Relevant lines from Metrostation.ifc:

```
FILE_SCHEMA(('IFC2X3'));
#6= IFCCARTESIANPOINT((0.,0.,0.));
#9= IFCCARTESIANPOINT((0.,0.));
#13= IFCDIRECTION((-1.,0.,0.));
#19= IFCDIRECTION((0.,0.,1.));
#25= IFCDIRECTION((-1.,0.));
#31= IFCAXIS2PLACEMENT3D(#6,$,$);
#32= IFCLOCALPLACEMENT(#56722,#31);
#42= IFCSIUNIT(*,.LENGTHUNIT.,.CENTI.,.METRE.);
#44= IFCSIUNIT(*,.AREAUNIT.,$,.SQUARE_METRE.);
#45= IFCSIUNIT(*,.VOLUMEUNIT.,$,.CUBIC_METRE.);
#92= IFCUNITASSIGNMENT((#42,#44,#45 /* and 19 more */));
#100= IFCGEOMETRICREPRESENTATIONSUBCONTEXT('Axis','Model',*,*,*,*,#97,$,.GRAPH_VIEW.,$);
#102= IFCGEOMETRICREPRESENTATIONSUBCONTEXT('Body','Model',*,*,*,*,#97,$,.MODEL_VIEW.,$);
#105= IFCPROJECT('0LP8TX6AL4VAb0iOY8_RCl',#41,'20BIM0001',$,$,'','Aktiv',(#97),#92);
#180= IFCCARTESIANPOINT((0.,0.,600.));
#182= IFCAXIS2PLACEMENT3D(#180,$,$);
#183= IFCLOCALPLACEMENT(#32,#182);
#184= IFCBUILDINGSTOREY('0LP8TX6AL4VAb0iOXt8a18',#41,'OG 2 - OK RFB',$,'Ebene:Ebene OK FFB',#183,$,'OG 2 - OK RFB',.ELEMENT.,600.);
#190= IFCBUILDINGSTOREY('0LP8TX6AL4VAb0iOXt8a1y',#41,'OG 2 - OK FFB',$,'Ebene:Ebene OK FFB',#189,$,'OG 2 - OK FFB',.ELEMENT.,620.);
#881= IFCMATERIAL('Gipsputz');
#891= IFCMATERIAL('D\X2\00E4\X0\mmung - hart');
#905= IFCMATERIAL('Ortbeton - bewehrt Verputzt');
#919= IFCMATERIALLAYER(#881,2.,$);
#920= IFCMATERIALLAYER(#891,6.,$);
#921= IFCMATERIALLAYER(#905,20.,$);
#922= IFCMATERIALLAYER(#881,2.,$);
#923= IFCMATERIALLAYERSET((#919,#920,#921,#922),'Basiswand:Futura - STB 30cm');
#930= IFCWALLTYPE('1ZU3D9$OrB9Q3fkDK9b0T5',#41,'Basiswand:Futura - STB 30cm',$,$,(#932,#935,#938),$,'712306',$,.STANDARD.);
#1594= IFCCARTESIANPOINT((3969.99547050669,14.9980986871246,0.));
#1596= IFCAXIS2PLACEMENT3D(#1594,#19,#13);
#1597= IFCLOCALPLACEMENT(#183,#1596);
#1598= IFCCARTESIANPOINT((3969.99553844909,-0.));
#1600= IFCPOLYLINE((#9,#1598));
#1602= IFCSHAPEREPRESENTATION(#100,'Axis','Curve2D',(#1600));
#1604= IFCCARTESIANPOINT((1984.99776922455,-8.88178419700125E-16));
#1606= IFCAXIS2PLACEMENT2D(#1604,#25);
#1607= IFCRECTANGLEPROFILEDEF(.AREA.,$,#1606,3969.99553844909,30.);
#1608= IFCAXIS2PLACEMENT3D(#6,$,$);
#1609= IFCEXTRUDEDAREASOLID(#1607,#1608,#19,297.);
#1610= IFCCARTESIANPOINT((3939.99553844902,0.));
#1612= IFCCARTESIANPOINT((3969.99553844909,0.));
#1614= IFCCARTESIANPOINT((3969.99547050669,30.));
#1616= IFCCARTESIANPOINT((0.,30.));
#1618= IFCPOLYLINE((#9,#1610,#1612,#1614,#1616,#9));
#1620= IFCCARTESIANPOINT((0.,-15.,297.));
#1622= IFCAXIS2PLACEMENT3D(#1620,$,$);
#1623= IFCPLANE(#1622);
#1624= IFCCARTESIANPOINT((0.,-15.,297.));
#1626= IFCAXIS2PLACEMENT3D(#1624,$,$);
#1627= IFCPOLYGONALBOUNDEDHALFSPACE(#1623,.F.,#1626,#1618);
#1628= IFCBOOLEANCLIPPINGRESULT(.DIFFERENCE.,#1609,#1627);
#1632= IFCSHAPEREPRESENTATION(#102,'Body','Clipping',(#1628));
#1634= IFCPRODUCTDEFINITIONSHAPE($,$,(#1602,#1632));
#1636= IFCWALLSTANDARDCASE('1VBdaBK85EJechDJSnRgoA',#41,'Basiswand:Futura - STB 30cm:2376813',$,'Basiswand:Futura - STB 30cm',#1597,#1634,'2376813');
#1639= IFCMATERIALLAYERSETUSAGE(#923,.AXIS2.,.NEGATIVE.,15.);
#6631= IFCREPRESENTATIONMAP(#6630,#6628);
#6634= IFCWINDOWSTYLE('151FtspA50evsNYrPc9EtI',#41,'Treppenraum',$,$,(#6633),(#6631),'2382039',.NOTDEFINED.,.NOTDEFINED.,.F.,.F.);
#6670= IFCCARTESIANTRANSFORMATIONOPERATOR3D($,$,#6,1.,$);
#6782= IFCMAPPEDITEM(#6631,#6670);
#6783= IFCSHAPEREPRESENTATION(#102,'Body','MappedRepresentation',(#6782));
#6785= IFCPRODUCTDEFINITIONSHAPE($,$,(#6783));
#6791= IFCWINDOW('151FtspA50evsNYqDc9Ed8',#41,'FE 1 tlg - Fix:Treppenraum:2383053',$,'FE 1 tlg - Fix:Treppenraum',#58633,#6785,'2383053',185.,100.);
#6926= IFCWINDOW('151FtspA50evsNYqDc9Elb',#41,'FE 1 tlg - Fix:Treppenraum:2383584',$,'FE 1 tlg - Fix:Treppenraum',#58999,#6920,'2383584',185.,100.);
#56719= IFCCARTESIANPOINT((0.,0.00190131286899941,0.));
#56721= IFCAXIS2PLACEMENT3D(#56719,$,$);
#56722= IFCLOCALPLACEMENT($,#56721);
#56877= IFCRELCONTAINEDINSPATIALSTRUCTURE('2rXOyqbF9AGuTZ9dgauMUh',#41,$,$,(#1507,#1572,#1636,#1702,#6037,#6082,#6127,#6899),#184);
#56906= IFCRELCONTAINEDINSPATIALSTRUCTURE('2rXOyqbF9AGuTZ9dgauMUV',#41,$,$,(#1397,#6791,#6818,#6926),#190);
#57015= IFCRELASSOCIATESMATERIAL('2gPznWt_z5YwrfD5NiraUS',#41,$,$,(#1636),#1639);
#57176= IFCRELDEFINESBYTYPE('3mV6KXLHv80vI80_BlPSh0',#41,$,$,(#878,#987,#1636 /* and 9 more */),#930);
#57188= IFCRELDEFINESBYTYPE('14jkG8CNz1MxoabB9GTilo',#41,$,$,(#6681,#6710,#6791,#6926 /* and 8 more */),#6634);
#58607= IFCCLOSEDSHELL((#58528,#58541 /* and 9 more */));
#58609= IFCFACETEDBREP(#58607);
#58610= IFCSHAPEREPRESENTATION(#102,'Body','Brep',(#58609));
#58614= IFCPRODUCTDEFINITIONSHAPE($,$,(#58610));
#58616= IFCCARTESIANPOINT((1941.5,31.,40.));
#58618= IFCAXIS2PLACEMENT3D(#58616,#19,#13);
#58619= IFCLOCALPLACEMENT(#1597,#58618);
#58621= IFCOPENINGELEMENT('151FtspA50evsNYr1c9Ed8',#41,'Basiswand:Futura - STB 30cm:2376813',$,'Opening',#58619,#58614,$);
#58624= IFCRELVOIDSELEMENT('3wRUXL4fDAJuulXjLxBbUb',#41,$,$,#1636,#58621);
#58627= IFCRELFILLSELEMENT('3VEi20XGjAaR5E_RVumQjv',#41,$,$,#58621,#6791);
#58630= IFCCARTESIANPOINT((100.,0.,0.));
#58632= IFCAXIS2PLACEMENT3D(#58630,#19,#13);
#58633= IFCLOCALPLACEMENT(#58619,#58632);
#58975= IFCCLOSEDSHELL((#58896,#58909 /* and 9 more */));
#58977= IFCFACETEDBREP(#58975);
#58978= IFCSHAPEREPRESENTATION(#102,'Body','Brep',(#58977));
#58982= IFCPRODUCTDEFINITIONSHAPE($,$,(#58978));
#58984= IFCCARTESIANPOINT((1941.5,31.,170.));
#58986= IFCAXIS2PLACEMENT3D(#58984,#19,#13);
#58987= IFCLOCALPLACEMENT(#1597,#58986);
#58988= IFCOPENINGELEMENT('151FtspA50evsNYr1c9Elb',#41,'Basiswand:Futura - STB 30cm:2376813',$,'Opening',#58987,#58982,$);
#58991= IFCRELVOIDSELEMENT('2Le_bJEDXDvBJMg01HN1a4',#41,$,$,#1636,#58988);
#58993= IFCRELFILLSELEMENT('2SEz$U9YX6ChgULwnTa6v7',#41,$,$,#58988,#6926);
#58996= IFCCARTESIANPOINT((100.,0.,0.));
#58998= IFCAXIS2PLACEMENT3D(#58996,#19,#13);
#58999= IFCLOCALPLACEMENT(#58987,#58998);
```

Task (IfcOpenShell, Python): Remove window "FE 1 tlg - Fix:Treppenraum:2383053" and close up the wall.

```python
import ifcopenshell
import ifcopenshell.api.feature
import ifcopenshell.api.root
import ifcopenshell.geom
import ifcopenshell.util.shape

model = ifcopenshell.open("Metrostation.ifc")
settings = ifcopenshell.geom.settings()


def volume(element):
    """Net volume in cubic metres, openings subtracted."""
    shape = ifcopenshell.geom.create_shape(settings, element)
    return ifcopenshell.util.shape.get_volume(shape.geometry)


window = model.by_guid("151FtspA50evsNYqDc9Ed8")
opening = window.FillsVoids[0].RelatingOpeningElement
wall = opening.VoidsElements[0].RelatingBuildingElement
before = volume(wall)

ifcopenshell.api.root.remove_product(model, product=window)
ifcopenshell.api.feature.remove_feature(model, feature=opening)

after = volume(wall)

print(f"wall volume {before:.3f} -> {after:.3f} m3")

model.write("Metrostation_edited.ifc")
```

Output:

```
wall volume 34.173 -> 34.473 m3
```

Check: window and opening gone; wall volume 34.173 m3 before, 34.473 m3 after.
